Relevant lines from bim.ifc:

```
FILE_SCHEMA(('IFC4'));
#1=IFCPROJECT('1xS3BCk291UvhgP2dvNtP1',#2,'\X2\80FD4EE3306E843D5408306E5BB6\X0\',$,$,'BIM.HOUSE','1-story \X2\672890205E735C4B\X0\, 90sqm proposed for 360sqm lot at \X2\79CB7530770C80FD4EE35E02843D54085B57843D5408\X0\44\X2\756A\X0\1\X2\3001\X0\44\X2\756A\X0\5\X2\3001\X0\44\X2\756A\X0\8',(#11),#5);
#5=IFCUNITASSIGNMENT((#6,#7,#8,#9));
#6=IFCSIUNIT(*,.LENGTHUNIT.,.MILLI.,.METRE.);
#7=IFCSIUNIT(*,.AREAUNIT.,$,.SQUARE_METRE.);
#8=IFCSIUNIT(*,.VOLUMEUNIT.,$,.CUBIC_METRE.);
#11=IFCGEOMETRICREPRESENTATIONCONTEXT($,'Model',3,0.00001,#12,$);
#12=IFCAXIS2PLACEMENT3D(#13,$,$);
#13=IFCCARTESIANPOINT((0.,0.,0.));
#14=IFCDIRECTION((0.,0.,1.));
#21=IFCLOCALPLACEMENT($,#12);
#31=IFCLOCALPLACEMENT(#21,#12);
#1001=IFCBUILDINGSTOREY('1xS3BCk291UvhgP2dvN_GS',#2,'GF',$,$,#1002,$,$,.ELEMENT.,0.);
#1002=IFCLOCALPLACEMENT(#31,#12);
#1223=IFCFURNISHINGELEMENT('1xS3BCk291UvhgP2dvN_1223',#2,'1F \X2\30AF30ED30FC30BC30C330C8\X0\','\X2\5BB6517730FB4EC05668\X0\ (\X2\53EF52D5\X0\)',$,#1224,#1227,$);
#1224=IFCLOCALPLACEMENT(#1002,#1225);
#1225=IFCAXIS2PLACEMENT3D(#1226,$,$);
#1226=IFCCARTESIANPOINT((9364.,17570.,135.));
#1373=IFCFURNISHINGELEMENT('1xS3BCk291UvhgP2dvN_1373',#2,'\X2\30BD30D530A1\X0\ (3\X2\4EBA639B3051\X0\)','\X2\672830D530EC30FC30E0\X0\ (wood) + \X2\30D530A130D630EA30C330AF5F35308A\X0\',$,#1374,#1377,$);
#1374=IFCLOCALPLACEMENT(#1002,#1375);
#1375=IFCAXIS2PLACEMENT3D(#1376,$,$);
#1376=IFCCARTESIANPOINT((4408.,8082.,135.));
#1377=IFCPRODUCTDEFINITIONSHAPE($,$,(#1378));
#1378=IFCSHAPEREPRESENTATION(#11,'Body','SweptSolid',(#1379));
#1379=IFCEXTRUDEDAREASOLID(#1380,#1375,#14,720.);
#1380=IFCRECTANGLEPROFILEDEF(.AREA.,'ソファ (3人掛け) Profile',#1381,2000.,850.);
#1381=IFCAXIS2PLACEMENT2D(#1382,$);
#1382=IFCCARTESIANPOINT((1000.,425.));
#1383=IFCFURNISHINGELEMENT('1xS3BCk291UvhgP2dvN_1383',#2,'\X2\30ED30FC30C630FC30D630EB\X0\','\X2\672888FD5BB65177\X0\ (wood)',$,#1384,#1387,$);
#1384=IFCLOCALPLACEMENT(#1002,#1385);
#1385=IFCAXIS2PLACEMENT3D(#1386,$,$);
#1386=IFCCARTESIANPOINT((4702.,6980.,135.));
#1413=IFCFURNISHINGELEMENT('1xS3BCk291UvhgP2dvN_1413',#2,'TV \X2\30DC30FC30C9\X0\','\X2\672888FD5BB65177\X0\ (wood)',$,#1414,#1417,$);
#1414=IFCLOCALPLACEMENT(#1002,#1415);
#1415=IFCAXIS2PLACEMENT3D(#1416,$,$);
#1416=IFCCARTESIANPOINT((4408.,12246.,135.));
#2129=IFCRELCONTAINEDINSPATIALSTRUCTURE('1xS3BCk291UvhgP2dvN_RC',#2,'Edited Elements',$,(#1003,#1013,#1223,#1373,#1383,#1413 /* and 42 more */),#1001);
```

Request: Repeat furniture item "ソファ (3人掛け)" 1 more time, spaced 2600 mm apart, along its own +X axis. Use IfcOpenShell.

```python
import ifcopenshell
import ifcopenshell.api.geometry
import ifcopenshell.api.root
import ifcopenshell.util.element
import ifcopenshell.util.placement
import ifcopenshell.util.unit

model = ifcopenshell.open("bim.ifc")
unit_scale = ifcopenshell.util.unit.calculate_unit_scale(model)


def reuse_history(source, copy):
    """copy_class also copies each property set's owner history, people and application; keep the originals."""
    for rel in copy.IsDefinedBy:
        if rel.is_a("IfcRelDefinesByProperties") and (history := rel.RelatingPropertyDefinition.OwnerHistory):
            rel.RelatingPropertyDefinition.OwnerHistory = source.OwnerHistory
            ifcopenshell.util.element.remove_deep2(model, history)


source = model.by_guid("1xS3BCk291UvhgP2dvN_1373")
base = ifcopenshell.util.placement.get_local_placement(source.ObjectPlacement)
step = base[:3, 0] * 2.6 / unit_scale

for i in range(1, 2):
    copy = ifcopenshell.api.root.copy_class(model, product=source)
    copy.Representation = ifcopenshell.util.element.copy_deep(
        model, source.Representation, exclude=["IfcGeometricRepresentationContext", "IfcRepresentationMap"]
    )
    reuse_history(source, copy)
    matrix = base.copy()
    matrix[:3, 3] += i * step
    print("added at", matrix[:3, 3].round(3) + 0.0)
    ifcopenshell.api.geometry.edit_object_placement(model, product=copy, matrix=matrix, is_si=False)

model.write("bim_edited.ifc")
```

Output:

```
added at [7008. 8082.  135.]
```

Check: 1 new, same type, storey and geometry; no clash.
